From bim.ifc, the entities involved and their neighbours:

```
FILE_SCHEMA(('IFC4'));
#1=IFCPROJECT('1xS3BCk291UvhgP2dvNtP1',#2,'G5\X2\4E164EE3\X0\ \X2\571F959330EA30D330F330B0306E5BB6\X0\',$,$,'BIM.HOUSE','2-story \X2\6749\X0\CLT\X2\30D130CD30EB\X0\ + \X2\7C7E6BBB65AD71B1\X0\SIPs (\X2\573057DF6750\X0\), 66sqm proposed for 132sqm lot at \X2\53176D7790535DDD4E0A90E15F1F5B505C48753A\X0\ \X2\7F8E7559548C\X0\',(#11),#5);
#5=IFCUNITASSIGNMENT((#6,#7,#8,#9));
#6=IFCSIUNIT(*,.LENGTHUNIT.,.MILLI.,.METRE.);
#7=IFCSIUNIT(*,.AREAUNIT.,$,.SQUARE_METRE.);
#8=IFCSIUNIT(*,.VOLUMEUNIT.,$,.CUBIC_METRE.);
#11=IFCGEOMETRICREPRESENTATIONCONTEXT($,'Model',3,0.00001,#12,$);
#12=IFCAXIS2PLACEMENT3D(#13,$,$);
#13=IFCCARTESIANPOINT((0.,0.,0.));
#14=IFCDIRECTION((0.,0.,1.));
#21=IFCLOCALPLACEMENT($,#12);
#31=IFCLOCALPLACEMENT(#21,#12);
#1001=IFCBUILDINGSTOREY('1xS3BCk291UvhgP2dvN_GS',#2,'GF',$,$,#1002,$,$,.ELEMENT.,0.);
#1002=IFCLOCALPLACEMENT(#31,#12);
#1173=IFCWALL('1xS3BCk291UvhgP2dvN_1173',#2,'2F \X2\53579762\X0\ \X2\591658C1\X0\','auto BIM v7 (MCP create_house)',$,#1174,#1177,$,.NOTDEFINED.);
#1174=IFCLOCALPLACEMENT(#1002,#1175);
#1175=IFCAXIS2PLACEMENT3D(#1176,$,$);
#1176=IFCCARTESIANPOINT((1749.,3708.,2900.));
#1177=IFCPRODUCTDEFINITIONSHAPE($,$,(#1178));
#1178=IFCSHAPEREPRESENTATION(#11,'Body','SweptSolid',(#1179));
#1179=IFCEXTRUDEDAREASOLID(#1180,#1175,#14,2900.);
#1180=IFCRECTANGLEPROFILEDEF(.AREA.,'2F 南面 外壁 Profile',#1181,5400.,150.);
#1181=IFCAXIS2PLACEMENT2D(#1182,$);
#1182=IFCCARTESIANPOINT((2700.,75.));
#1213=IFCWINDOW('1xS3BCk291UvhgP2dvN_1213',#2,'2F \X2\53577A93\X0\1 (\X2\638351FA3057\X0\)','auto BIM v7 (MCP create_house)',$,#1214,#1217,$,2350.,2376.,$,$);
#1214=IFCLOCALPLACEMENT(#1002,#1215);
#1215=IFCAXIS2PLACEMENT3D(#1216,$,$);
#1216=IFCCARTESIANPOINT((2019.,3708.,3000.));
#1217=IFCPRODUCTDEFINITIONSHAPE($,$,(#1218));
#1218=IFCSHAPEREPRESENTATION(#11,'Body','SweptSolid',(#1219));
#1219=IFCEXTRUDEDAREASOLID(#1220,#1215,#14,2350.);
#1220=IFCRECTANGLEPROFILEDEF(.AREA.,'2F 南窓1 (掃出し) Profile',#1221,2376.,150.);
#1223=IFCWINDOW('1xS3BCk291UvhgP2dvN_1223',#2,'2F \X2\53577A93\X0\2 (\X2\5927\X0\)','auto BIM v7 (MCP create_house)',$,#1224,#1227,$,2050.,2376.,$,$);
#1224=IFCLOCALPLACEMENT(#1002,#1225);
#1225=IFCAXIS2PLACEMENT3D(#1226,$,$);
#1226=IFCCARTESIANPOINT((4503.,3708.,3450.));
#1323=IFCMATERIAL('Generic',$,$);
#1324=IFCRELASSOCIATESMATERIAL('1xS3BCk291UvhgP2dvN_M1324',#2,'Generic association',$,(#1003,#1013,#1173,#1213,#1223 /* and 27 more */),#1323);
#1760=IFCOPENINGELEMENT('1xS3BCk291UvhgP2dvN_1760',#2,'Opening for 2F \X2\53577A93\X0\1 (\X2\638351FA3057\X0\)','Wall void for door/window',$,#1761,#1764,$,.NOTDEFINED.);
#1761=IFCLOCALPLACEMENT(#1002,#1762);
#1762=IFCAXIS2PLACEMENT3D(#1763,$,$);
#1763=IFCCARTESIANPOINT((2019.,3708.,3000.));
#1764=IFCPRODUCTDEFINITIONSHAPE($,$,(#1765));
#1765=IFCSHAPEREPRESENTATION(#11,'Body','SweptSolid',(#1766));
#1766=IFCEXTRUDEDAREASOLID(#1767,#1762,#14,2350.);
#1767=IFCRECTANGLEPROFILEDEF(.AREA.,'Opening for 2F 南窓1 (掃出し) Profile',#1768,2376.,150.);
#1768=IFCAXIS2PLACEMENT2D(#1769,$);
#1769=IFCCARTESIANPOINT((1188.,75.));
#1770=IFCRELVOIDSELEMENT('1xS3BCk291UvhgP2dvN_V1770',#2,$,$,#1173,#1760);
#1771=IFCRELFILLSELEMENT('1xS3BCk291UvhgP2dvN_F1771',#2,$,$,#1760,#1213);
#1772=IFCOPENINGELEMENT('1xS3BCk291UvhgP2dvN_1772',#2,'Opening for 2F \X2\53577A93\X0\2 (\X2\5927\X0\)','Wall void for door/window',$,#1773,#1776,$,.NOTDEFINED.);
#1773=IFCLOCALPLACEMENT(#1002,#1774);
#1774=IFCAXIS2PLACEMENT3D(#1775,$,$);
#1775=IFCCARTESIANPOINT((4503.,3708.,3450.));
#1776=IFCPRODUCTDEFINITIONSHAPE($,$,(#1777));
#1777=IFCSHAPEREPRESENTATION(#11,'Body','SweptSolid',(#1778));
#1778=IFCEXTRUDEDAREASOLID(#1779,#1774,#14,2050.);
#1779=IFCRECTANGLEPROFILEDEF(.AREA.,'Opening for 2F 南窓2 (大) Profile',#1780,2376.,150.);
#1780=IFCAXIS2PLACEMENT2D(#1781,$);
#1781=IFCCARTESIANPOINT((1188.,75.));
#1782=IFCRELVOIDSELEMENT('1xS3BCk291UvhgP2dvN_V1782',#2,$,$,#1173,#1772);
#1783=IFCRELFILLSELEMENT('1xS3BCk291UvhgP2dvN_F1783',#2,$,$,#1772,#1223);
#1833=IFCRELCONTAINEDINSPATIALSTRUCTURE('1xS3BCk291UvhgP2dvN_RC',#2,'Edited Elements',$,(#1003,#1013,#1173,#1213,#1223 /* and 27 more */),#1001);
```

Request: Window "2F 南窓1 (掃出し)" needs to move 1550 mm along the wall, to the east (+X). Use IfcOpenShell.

```python
import ifcopenshell
import ifcopenshell.api.geometry
import ifcopenshell.util.placement
import ifcopenshell.util.unit

model = ifcopenshell.open("bim.ifc")
unit_scale = ifcopenshell.util.unit.calculate_unit_scale(model)

window = model.by_guid("1xS3BCk291UvhgP2dvN_1213")
opening = window.FillsVoids[0].RelatingOpeningElement
wall = opening.VoidsElements[0].RelatingBuildingElement

wall_matrix = ifcopenshell.util.placement.get_local_placement(wall.ObjectPlacement)
shift = wall_matrix[:3, 0] * 1.55 / unit_scale
before = ifcopenshell.util.placement.get_local_placement(window.ObjectPlacement)[:3, 3].copy()

# The window is not placed relative to its opening, so move both.
for product in (opening, window):
    matrix = ifcopenshell.util.placement.get_local_placement(product.ObjectPlacement)
    matrix[:3, 3] += shift
    ifcopenshell.api.geometry.edit_object_placement(model, product=product, matrix=matrix, is_si=False)

after = ifcopenshell.util.placement.get_local_placement(window.ObjectPlacement)[:3, 3]
print("window moved by", (after - before).round(3) + 0.0)

model.write("bim_edited.ifc")
```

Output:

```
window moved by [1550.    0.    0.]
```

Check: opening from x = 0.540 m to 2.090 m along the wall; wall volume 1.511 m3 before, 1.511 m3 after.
